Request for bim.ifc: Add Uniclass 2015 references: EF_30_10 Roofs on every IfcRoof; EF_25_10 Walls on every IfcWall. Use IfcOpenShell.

First a look at what the model holds.

```python
import ifcopenshell

model = ifcopenshell.open("bim.ifc")
print(model.schema)
print("classifications:", [c.Name for c in model.by_type("IfcClassification")])
for ifc_class in ("IfcDoor", "IfcRoof", "IfcStair", "IfcWall", "IfcWindow"):
    print(ifc_class, len(model.by_type(ifc_class)))
```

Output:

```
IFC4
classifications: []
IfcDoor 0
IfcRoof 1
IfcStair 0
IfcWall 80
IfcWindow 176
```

```python
import ifcopenshell
import ifcopenshell.api.classification

model = ifcopenshell.open("bim.ifc")

system = ifcopenshell.api.classification.add_classification(model, classification="Uniclass 2015")

codes = {
    "IfcRoof": ("EF_30_10", "Roofs"),
    "IfcWall": ("EF_25_10", "Walls"),
}
for ifc_class, (code, name) in codes.items():
    products = model.by_type(ifc_class)
    ifcopenshell.api.classification.add_reference(
        model, products=products, classification=system, identification=code, name=name
    )
    print(code, len(products))

model.write("bim_edited.ifc")
```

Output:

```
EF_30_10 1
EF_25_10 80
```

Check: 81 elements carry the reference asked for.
